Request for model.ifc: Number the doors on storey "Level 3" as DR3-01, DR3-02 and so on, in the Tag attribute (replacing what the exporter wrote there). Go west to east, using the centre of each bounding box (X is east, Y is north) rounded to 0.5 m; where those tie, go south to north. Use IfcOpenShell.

First a look at what the model holds.

```python
import ifcopenshell
import ifcopenshell.util.element
import ifcopenshell.util.placement

model = ifcopenshell.open("model.ifc")
print(model.schema)
storey = next(s for s in model.by_type("IfcBuildingStorey") if s.Name == "Level 3")
doors = [e for e in ifcopenshell.util.element.get_decomposition(storey) if e.is_a("IfcDoor")]
for e in sorted(doors, key=lambda e: e.id()):
    origin = ifcopenshell.util.placement.get_local_placement(e.ObjectPlacement)[:3, 3]
    print(e.id(), e.Tag, e.Name, origin.round(2) + 0.0, sep=" | ")
```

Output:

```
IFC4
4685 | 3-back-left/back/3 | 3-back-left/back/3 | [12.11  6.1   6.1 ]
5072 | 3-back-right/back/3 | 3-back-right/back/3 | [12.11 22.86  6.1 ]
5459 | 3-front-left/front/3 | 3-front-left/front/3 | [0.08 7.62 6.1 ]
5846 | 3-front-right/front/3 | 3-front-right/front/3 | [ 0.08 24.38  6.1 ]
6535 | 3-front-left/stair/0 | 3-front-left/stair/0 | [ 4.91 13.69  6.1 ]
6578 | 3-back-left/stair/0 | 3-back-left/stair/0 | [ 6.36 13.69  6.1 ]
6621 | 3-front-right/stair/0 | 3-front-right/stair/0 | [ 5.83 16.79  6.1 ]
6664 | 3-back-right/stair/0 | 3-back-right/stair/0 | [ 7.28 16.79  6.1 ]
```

```python
import ifcopenshell
import ifcopenshell.geom
import ifcopenshell.util.element
import ifcopenshell.util.shape

model = ifcopenshell.open("model.ifc")
settings = ifcopenshell.geom.settings()
settings.set("use-world-coords", True)


def centre(element):
    shape = ifcopenshell.geom.create_shape(settings, element)
    return ifcopenshell.util.shape.get_bbox_centroid(shape.geometry)


storey = next(s for s in model.by_type("IfcBuildingStorey") if s.Name == "Level 3")
doors = [e for e in ifcopenshell.util.element.get_decomposition(storey) if e.is_a("IfcDoor")]

# Insertion points can sit at a corner or the storey origin, so sort by the geometry (in metres).
centres = {e: centre(e) for e in doors}
doors.sort(key=lambda e: (round(centres[e][0] / 0.5), centres[e][1]))

for i, e in enumerate(doors, start=1):
    number = f"DR3-{i:02d}"
    e.Tag = number
    print(e.id(), number)

model.write("model_rev.ifc")
```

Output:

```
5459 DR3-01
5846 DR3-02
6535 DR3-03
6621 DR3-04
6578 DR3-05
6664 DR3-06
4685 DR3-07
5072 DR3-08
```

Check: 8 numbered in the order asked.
